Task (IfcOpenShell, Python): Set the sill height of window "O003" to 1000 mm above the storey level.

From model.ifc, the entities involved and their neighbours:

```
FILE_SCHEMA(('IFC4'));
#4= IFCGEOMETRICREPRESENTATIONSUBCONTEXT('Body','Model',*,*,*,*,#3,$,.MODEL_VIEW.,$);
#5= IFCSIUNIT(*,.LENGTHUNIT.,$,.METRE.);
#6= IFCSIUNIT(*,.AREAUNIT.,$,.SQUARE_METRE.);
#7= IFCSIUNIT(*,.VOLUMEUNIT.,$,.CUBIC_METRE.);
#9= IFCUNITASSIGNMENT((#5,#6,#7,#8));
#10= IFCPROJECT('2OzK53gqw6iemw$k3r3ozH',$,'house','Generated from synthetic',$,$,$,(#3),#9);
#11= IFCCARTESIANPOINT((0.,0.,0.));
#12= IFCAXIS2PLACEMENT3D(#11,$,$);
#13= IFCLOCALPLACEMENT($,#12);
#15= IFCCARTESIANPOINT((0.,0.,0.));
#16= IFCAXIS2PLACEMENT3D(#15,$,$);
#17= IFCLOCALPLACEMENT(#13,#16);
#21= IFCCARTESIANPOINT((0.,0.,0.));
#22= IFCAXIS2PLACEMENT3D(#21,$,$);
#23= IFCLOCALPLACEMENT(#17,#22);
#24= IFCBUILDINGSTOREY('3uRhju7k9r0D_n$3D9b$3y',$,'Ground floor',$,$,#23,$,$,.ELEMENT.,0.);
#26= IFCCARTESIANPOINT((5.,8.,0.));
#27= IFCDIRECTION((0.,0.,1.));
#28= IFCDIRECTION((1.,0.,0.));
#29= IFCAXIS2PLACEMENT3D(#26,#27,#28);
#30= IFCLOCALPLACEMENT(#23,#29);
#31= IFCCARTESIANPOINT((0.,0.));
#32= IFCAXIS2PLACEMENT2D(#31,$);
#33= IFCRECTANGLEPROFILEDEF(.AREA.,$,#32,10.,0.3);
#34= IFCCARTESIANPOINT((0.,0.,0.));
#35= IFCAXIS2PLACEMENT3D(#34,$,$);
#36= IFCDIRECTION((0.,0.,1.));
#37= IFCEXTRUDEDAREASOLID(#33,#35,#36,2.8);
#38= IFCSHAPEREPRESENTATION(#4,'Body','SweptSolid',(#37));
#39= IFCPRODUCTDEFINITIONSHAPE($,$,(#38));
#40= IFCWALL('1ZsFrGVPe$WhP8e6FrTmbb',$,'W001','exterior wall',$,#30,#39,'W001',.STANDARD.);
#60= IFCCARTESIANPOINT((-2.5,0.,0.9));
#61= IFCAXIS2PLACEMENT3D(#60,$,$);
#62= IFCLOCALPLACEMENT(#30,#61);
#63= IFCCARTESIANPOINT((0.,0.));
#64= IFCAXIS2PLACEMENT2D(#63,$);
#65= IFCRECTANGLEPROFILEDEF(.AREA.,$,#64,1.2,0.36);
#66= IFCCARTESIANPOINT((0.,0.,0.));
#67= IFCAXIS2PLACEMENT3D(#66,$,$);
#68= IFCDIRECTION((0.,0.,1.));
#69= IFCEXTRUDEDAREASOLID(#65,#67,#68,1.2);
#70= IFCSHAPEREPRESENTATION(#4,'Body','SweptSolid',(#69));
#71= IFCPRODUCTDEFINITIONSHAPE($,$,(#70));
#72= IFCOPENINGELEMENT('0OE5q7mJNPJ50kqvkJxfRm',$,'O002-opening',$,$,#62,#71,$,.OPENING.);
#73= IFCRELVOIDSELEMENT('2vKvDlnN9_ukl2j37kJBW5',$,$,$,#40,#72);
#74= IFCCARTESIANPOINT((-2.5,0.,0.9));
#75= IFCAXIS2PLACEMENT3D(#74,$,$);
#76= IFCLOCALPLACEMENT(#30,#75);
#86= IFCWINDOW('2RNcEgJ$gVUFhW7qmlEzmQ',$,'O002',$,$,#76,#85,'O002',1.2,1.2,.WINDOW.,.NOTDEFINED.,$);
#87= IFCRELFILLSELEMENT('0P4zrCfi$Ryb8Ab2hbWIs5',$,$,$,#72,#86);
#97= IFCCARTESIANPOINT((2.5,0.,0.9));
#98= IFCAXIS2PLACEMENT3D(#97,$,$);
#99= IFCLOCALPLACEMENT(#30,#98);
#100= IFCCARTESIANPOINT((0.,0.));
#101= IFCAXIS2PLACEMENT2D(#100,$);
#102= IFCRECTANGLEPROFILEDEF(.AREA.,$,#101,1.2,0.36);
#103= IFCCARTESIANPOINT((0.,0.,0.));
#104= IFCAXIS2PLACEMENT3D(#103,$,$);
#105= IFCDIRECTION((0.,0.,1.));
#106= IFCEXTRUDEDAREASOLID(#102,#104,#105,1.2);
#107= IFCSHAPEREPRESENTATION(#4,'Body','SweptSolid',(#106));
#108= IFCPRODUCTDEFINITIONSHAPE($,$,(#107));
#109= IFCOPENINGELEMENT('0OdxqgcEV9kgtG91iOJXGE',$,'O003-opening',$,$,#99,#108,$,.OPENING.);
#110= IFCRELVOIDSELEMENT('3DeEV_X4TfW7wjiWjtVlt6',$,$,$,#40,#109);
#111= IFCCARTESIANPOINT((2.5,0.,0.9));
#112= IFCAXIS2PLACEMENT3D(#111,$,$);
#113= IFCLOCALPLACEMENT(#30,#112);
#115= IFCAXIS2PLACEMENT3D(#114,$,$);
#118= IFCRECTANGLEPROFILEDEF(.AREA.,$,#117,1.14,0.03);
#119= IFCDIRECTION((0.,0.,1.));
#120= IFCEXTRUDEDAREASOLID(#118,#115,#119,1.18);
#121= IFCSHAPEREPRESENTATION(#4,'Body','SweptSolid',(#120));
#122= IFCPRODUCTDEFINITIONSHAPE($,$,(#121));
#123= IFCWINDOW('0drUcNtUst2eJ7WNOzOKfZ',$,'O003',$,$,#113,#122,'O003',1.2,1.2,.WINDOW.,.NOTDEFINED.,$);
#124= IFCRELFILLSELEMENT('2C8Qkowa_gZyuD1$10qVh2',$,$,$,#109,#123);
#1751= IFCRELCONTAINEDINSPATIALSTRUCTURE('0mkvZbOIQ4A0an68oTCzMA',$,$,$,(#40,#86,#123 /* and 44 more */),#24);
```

```python
import numpy as np
import ifcopenshell
import ifcopenshell.api.geometry
import ifcopenshell.geom
import ifcopenshell.util.element
import ifcopenshell.util.placement
import ifcopenshell.util.shape
import ifcopenshell.util.unit

model = ifcopenshell.open("model.ifc")
unit_scale = ifcopenshell.util.unit.calculate_unit_scale(model)

window = model.by_guid("0drUcNtUst2eJ7WNOzOKfZ")
opening = window.FillsVoids[0].RelatingOpeningElement
storey = ifcopenshell.util.element.get_container(window, ifc_class="IfcBuildingStorey")
level = ifcopenshell.util.placement.get_local_placement(storey.ObjectPlacement)[2, 3]

# The opening's origin need not be at the sill, so measure its lowest point.
shape = ifcopenshell.geom.create_shape(ifcopenshell.geom.settings(), opening)
bottom = ifcopenshell.util.shape.get_shape_bottom_elevation(shape, shape.geometry) / unit_scale
dz = level + 1 / unit_scale - bottom

shift = np.array([0.0, 0.0, dz])
# The window is not placed relative to its opening, so move both.
for product in (opening, window):
    matrix = ifcopenshell.util.placement.get_local_placement(product.ObjectPlacement)
    matrix[:3, 3] += shift
    ifcopenshell.api.geometry.edit_object_placement(model, product=product, matrix=matrix, is_si=False)

print(f"moved by {dz * unit_scale:+.3f} m")

model.write("model_updated.ifc")
```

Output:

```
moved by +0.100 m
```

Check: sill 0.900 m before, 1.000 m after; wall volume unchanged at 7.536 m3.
